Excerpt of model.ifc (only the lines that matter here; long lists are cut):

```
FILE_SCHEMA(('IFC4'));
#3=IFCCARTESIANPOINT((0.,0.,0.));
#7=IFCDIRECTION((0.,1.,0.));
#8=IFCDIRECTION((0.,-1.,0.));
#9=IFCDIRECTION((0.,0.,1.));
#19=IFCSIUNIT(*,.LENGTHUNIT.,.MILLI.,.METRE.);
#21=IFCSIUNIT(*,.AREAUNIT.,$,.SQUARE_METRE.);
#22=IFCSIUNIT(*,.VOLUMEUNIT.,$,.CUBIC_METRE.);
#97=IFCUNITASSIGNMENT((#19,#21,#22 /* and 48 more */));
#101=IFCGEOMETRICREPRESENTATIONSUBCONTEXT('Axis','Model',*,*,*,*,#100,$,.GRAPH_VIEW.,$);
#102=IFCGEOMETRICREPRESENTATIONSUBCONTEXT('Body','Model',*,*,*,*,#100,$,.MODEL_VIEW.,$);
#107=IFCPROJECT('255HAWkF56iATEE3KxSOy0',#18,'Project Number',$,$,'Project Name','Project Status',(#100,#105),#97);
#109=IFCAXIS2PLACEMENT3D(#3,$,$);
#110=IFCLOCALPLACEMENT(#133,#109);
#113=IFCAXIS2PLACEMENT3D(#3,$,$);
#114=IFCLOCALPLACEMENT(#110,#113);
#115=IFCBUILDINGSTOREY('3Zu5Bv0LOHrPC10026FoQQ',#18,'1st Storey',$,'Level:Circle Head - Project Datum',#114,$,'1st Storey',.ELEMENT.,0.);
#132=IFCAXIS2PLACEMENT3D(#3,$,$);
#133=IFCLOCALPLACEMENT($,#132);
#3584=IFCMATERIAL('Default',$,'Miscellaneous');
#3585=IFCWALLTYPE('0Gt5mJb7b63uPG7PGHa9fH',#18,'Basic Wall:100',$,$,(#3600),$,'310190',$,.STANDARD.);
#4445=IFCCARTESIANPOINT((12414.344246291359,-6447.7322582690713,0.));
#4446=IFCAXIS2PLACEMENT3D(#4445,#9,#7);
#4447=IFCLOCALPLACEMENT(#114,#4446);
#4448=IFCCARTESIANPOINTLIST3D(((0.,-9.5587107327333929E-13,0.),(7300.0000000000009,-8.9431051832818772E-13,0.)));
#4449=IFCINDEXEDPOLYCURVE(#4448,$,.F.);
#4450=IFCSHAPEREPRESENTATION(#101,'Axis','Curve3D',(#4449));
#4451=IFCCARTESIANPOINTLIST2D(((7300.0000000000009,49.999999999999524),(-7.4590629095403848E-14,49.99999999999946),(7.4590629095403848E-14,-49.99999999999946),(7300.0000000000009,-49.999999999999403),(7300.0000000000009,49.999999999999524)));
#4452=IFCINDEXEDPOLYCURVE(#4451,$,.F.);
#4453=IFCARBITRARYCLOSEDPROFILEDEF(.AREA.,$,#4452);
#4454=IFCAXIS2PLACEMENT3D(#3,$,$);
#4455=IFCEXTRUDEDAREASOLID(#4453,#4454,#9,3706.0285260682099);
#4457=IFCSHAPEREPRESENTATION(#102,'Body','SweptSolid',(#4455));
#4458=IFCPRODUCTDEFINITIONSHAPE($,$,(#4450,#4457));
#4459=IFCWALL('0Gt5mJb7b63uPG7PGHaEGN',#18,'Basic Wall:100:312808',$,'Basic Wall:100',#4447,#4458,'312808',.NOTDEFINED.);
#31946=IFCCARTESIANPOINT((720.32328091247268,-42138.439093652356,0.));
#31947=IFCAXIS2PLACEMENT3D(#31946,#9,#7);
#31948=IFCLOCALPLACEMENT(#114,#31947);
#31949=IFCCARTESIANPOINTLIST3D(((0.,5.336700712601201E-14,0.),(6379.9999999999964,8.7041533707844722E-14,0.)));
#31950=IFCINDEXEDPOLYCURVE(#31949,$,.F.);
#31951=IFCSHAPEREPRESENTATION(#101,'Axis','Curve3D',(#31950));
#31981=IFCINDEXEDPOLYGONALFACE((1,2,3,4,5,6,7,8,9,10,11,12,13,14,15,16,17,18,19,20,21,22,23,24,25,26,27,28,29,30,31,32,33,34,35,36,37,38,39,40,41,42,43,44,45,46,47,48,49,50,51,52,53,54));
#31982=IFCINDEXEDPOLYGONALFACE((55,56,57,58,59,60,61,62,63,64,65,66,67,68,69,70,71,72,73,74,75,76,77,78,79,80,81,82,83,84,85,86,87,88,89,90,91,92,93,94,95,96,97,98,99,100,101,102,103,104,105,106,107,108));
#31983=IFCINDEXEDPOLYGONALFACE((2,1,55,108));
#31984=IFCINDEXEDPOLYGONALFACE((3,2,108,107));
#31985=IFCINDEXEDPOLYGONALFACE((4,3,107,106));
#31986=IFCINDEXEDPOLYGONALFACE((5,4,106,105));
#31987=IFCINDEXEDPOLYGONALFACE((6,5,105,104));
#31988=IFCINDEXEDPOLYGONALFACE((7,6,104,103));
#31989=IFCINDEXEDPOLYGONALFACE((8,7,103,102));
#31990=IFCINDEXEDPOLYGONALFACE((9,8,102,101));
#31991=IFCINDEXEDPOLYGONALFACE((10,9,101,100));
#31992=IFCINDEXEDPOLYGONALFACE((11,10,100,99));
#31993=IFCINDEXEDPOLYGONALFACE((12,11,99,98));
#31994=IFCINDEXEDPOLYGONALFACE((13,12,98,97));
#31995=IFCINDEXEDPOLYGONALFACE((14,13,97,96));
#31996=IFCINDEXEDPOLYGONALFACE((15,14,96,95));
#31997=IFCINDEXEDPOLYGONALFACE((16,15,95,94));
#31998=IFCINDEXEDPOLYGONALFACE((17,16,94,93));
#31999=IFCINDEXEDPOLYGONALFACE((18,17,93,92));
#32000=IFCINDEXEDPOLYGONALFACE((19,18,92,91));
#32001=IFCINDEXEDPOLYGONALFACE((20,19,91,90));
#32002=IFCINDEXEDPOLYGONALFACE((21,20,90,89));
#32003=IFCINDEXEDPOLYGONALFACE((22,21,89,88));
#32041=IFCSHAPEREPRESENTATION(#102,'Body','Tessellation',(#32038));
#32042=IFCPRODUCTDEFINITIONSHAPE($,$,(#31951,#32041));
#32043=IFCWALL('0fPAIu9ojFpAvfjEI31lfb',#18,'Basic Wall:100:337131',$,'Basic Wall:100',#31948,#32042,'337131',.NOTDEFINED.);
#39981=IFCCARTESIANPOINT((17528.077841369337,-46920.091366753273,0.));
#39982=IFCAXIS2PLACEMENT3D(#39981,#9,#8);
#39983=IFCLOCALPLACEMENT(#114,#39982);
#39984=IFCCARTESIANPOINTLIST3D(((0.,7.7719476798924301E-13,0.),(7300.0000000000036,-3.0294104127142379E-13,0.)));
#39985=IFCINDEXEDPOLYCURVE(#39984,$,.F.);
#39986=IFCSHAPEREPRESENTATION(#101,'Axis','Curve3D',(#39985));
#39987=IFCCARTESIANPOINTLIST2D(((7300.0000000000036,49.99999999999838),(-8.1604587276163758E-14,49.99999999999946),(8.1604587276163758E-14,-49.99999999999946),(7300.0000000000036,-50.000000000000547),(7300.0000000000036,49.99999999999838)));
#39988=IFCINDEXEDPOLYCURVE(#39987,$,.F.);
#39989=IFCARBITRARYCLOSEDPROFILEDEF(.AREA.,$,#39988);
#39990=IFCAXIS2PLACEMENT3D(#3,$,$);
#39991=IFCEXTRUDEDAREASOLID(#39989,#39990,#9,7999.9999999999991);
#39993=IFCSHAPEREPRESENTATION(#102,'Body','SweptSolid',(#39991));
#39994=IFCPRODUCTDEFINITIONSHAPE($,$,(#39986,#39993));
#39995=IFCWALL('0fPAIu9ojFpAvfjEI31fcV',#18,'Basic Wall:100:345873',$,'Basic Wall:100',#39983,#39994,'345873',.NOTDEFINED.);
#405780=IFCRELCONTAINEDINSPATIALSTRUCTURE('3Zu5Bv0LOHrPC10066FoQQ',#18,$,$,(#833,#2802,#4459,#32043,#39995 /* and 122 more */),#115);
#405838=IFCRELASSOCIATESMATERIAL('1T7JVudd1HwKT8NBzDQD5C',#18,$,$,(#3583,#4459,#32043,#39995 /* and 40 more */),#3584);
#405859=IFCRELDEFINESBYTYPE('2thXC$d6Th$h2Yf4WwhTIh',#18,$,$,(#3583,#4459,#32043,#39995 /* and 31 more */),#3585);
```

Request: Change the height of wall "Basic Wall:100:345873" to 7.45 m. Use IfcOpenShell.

```python
import ifcopenshell
import ifcopenshell.geom
import ifcopenshell.util.representation
import ifcopenshell.util.shape
import ifcopenshell.util.unit

model = ifcopenshell.open("model.ifc")
unit_scale = ifcopenshell.util.unit.calculate_unit_scale(model)
settings = ifcopenshell.geom.settings()


def volume(element):
    """Net volume in cubic metres, openings subtracted."""
    shape = ifcopenshell.geom.create_shape(settings, element)
    return ifcopenshell.util.shape.get_volume(shape.geometry)


wall = model.by_id(39995)
before = volume(wall)

body = ifcopenshell.util.representation.get_representation(wall, "Model", "Body")
solid = body.Items[0]
old_height = solid.Depth
solid.Depth = 7.45 / unit_scale
after = volume(wall)

print(f"height {old_height:g} -> {solid.Depth:g}, volume {before:.3f} -> {after:.3f} m3")

model.write("model_updated.ifc")
```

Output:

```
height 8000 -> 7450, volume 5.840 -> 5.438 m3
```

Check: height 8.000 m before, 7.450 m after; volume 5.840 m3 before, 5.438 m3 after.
